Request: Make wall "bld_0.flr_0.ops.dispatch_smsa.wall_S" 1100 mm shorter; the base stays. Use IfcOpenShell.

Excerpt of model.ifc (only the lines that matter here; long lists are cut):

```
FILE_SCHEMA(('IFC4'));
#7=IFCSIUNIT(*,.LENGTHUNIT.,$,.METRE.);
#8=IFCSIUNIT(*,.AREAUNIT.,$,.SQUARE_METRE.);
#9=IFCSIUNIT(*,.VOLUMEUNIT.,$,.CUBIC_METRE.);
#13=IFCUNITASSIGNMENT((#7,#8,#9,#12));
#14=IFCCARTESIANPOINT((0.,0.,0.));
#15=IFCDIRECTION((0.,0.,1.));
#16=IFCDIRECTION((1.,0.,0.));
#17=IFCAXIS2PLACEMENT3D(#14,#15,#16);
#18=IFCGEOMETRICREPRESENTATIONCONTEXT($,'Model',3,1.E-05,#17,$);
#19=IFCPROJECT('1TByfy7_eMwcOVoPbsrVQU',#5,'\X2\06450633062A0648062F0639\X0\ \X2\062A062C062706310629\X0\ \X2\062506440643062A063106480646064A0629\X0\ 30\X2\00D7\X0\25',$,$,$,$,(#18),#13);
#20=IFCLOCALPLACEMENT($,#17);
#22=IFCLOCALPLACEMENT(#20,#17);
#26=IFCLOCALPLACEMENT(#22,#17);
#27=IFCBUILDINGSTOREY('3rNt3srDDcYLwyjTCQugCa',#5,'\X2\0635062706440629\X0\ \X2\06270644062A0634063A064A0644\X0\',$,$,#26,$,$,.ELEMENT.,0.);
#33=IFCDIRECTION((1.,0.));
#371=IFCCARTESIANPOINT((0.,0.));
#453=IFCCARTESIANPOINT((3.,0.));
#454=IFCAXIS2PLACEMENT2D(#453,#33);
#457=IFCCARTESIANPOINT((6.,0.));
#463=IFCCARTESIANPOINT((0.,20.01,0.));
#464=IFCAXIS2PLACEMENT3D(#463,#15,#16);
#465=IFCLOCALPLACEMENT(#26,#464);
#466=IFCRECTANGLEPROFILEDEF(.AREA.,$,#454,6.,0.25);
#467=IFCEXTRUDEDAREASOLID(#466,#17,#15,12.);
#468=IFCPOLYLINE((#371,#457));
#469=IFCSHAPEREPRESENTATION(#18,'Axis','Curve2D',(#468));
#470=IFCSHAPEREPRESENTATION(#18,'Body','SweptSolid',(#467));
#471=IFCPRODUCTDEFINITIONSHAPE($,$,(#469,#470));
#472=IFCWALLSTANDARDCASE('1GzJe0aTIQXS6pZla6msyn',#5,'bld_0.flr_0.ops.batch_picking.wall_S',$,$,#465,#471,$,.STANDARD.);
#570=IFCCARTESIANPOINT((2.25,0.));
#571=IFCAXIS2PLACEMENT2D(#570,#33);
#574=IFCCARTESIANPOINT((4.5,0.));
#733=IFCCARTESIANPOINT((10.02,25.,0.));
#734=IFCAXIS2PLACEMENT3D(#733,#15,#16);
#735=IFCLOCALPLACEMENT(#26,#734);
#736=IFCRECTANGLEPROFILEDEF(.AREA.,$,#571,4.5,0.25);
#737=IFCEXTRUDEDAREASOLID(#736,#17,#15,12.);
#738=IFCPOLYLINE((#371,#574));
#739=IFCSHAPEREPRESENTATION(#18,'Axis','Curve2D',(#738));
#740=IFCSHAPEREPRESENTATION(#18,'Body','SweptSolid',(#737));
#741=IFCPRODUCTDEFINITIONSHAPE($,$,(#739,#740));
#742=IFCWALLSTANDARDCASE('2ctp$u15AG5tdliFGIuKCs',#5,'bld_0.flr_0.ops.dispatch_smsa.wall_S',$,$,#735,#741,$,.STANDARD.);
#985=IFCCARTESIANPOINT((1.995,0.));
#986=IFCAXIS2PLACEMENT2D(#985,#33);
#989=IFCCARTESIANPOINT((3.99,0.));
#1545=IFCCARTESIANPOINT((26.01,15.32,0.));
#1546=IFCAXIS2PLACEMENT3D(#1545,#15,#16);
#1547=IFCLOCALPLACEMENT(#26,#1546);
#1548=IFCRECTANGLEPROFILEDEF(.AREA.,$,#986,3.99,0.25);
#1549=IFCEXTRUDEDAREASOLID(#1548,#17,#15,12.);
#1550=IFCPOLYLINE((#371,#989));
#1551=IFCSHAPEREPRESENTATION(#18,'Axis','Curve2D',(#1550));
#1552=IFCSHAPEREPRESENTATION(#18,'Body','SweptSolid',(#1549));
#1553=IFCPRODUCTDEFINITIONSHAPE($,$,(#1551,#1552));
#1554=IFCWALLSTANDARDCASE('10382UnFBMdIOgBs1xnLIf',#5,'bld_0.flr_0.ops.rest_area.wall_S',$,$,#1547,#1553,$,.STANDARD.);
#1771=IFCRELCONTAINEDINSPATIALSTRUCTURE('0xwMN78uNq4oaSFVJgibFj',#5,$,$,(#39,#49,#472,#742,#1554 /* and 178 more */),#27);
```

```python
import ifcopenshell
import ifcopenshell.geom
import ifcopenshell.util.shape
import ifcopenshell.util.unit

model = ifcopenshell.open("model.ifc")
unit_scale = ifcopenshell.util.unit.calculate_unit_scale(model)
settings = ifcopenshell.geom.settings()


def volume(element):
    """Net volume in cubic metres, openings subtracted."""
    shape = ifcopenshell.geom.create_shape(settings, element)
    return ifcopenshell.util.shape.get_volume(shape.geometry)


wall = model.by_guid("2ctp$u15AG5tdliFGIuKCs")
before = volume(wall)

body = next(r for r in wall.Representation.Representations if r.RepresentationIdentifier == "Body")
solid = body.Items[0]
old_height = solid.Depth
solid.Depth -= 1.1 / unit_scale
after = volume(wall)

print(f"height {old_height:g} -> {solid.Depth:g}, volume {before:.3f} -> {after:.3f} m3")

model.write("model_rev.ifc")
```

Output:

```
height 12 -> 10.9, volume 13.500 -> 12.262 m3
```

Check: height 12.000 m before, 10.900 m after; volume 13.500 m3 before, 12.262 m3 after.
